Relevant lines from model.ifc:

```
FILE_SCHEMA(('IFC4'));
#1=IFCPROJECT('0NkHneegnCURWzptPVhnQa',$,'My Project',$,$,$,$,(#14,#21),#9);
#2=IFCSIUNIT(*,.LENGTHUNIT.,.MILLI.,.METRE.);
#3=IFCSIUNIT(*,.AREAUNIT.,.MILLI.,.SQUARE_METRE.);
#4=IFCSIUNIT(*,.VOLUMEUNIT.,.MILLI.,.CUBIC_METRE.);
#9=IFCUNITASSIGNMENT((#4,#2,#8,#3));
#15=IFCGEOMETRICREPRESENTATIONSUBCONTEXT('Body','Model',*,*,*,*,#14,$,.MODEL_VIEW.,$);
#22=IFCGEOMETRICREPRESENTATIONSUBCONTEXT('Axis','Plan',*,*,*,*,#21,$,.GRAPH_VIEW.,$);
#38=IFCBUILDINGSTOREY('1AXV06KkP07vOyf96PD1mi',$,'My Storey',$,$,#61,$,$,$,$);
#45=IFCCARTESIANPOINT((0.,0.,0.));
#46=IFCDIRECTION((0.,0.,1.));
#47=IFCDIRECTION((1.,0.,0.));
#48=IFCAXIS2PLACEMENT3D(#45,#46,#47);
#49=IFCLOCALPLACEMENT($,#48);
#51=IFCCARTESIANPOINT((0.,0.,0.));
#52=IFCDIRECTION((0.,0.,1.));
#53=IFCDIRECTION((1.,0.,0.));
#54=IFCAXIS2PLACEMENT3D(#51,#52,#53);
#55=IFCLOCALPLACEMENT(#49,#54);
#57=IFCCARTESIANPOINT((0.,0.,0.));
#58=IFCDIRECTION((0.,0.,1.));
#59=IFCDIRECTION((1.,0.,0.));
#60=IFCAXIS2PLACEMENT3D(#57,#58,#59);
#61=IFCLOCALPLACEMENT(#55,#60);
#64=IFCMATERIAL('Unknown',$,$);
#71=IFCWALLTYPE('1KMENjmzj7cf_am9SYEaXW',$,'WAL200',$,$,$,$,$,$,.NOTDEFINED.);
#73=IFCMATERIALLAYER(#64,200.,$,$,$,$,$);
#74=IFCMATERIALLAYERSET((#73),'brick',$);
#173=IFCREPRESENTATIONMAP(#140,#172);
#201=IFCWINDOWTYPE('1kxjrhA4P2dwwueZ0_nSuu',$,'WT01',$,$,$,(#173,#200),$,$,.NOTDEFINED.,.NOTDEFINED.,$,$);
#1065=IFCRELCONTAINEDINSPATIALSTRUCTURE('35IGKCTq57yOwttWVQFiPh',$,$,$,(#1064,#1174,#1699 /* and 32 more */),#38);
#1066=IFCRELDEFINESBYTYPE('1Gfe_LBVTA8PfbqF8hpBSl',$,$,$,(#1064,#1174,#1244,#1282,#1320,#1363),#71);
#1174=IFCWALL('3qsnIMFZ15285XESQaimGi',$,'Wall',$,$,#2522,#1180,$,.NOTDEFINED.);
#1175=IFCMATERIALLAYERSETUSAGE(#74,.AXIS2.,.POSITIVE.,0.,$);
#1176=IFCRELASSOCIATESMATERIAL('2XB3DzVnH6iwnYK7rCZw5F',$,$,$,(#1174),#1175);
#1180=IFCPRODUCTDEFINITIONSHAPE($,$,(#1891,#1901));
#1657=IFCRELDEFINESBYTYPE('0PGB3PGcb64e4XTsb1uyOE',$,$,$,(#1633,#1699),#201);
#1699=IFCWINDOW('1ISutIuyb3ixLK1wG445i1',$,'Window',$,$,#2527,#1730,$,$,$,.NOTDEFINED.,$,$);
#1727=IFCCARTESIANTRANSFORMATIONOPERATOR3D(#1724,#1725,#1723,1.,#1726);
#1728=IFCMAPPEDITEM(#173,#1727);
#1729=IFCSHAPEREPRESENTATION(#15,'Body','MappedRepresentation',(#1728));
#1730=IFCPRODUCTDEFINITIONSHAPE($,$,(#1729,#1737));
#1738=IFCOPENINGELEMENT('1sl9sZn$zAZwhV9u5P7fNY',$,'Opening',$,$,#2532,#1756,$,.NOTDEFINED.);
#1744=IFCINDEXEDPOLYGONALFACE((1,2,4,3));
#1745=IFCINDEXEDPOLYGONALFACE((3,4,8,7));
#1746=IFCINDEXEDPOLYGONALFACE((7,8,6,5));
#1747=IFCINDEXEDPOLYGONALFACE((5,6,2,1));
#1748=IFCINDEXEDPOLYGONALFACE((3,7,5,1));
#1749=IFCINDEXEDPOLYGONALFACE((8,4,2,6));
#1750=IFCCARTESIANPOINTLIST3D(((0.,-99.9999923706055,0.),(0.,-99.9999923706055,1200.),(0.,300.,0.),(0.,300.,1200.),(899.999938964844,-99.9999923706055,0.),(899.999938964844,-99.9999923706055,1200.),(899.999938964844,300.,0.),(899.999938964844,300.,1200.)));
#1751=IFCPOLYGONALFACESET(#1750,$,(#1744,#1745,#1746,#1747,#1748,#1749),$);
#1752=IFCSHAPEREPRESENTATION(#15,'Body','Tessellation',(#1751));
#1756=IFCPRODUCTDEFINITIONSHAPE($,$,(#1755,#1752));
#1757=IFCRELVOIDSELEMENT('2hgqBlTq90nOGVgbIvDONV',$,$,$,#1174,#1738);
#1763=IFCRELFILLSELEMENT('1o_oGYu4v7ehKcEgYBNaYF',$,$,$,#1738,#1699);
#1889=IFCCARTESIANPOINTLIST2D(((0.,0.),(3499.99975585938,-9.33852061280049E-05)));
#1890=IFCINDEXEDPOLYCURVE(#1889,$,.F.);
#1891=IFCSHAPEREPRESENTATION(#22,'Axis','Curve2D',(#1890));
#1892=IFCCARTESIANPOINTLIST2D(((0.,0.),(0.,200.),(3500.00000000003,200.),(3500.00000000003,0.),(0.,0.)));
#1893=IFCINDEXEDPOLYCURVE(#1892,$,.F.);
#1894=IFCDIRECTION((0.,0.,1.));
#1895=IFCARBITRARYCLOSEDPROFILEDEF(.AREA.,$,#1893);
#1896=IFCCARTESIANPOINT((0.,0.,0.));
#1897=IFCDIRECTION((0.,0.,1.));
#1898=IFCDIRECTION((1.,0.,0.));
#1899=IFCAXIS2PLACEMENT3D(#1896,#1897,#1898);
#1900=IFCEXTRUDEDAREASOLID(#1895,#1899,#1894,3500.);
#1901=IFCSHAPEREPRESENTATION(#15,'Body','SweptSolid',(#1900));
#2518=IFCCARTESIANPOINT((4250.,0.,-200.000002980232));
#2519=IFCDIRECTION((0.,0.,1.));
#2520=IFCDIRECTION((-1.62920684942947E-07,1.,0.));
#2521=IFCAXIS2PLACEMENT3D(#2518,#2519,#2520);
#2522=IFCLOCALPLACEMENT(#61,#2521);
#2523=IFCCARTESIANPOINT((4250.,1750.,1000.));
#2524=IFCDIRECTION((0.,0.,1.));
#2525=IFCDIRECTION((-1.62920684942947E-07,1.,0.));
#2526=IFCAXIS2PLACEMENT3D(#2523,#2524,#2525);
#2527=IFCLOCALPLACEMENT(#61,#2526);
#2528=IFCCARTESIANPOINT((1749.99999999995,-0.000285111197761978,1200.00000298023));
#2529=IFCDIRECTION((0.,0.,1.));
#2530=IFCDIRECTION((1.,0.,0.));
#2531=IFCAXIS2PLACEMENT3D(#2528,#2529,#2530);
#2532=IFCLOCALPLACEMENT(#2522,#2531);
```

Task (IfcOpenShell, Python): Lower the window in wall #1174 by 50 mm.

```python
import numpy as np
import ifcopenshell
import ifcopenshell.api.geometry
import ifcopenshell.util.placement
import ifcopenshell.util.unit

model = ifcopenshell.open("model.ifc")
unit_scale = ifcopenshell.util.unit.calculate_unit_scale(model)

window = model.by_guid("1ISutIuyb3ixLK1wG445i1")
opening = window.FillsVoids[0].RelatingOpeningElement
dz = -0.05 / unit_scale

shift = np.array([0.0, 0.0, dz])
# The window is not placed relative to its opening, so move both.
for product in (opening, window):
    matrix = ifcopenshell.util.placement.get_local_placement(product.ObjectPlacement)
    matrix[:3, 3] += shift
    ifcopenshell.api.geometry.edit_object_placement(model, product=product, matrix=matrix, is_si=False)

print(f"moved by {dz * unit_scale:+.3f} m")

model.write("model_updated.ifc")
```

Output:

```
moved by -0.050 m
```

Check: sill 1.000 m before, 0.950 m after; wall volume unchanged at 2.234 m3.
